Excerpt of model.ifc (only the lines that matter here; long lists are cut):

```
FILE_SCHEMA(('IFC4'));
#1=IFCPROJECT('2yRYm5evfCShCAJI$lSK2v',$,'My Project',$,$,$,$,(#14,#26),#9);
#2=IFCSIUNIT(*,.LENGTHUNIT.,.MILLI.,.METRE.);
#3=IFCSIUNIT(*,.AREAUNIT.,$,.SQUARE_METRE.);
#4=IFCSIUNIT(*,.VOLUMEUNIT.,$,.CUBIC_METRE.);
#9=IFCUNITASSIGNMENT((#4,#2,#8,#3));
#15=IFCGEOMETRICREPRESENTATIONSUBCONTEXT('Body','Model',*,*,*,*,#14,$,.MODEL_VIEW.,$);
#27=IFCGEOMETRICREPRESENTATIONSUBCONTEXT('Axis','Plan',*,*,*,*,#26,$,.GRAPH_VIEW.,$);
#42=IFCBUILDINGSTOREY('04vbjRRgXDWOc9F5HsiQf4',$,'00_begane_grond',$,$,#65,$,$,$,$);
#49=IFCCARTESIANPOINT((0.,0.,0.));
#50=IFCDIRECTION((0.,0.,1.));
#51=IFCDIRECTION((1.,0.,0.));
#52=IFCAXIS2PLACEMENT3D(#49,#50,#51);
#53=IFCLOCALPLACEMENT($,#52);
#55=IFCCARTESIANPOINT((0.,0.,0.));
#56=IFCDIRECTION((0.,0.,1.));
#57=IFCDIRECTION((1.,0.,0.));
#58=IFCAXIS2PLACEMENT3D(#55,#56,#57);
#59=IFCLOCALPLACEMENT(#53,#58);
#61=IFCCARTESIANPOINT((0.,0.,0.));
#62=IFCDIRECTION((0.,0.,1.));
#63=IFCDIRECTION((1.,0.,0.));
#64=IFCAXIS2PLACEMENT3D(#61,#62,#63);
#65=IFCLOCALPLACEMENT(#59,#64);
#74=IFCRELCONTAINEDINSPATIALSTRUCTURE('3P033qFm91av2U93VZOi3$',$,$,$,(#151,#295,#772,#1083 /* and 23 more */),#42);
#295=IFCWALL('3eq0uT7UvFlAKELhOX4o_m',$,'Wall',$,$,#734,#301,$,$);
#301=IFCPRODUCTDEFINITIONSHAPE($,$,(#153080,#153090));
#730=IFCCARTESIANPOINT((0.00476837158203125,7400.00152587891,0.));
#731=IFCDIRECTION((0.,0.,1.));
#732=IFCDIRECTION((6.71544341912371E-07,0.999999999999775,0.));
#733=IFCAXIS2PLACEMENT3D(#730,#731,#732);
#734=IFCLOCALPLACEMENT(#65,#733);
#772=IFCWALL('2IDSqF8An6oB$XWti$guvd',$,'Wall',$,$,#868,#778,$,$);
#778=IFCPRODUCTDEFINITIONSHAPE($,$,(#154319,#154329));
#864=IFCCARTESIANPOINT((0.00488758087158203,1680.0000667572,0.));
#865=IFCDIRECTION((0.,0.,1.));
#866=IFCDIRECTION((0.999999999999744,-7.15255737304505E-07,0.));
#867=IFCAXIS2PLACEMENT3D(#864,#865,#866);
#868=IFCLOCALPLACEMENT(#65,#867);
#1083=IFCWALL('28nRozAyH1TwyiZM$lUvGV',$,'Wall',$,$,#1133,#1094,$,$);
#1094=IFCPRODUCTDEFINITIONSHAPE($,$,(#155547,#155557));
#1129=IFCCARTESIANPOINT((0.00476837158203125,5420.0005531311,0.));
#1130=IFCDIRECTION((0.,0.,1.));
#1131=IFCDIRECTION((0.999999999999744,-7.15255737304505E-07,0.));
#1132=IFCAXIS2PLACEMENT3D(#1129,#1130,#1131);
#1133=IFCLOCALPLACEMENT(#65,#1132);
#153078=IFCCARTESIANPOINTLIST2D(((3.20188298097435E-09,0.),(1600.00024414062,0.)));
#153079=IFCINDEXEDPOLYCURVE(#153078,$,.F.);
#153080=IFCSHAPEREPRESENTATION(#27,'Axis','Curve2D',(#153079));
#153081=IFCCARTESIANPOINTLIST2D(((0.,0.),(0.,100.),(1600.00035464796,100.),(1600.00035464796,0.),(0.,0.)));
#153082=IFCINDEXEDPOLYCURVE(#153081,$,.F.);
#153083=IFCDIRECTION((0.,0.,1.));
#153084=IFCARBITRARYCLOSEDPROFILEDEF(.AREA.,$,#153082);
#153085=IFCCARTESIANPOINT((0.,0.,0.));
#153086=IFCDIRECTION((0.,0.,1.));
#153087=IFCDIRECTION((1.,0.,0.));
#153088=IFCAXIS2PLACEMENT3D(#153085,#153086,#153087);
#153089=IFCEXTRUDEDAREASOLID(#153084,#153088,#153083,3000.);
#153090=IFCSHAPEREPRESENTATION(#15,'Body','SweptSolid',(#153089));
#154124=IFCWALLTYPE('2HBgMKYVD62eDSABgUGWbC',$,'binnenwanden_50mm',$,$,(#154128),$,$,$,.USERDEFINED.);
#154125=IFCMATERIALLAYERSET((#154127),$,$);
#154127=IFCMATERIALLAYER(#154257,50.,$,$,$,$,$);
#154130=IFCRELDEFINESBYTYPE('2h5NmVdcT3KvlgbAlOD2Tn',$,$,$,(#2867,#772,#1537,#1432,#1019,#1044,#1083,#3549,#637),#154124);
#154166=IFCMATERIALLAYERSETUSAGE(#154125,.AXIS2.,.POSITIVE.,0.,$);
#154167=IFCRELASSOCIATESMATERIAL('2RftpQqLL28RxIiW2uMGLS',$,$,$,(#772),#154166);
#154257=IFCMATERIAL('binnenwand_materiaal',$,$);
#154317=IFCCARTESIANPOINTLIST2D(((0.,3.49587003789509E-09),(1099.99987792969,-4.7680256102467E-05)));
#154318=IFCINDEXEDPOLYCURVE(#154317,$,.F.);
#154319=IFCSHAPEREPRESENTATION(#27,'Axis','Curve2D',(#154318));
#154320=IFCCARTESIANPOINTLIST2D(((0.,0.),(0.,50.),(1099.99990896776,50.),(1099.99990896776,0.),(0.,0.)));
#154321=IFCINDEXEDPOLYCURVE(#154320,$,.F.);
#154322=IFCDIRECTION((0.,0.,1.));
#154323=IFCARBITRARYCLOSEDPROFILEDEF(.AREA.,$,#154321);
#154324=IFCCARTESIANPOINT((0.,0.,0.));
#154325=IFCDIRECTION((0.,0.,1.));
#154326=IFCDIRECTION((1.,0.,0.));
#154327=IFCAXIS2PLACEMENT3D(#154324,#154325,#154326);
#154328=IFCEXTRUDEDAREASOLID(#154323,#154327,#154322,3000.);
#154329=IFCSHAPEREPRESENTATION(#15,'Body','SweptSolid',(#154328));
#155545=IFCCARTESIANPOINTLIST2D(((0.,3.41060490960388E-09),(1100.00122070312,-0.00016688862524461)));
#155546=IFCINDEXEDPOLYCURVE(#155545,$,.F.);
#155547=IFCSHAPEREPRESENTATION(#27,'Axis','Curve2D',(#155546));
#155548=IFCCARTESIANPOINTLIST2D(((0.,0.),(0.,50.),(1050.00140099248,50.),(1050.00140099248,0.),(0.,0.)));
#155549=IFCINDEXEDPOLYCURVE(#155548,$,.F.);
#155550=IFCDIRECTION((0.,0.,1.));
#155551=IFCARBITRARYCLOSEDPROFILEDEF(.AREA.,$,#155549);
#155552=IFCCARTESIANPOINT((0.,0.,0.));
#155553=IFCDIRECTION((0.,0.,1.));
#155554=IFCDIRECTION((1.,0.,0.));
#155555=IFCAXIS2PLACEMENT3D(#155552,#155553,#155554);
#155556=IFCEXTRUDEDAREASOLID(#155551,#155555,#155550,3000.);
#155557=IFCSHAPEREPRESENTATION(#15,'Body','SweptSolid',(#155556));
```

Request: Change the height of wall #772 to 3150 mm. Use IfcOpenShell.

```python
import ifcopenshell
import ifcopenshell.geom
import ifcopenshell.util.representation
import ifcopenshell.util.shape
import ifcopenshell.util.unit

model = ifcopenshell.open("model.ifc")
unit_scale = ifcopenshell.util.unit.calculate_unit_scale(model)
settings = ifcopenshell.geom.settings()


def volume(element):
    """Net volume in cubic metres, openings subtracted."""
    shape = ifcopenshell.geom.create_shape(settings, element)
    return ifcopenshell.util.shape.get_volume(shape.geometry)


wall = model.by_id(772)
before = volume(wall)

body = ifcopenshell.util.representation.get_representation(wall, "Model", "Body")
solid = body.Items[0]
old_height = solid.Depth
solid.Depth = 3.15 / unit_scale
after = volume(wall)

print(f"height {old_height:g} -> {solid.Depth:g}, volume {before:.3f} -> {after:.3f} m3")

model.write("model-out.ifc")
```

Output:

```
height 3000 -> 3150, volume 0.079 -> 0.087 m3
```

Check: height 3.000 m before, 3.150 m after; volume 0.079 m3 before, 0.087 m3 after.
